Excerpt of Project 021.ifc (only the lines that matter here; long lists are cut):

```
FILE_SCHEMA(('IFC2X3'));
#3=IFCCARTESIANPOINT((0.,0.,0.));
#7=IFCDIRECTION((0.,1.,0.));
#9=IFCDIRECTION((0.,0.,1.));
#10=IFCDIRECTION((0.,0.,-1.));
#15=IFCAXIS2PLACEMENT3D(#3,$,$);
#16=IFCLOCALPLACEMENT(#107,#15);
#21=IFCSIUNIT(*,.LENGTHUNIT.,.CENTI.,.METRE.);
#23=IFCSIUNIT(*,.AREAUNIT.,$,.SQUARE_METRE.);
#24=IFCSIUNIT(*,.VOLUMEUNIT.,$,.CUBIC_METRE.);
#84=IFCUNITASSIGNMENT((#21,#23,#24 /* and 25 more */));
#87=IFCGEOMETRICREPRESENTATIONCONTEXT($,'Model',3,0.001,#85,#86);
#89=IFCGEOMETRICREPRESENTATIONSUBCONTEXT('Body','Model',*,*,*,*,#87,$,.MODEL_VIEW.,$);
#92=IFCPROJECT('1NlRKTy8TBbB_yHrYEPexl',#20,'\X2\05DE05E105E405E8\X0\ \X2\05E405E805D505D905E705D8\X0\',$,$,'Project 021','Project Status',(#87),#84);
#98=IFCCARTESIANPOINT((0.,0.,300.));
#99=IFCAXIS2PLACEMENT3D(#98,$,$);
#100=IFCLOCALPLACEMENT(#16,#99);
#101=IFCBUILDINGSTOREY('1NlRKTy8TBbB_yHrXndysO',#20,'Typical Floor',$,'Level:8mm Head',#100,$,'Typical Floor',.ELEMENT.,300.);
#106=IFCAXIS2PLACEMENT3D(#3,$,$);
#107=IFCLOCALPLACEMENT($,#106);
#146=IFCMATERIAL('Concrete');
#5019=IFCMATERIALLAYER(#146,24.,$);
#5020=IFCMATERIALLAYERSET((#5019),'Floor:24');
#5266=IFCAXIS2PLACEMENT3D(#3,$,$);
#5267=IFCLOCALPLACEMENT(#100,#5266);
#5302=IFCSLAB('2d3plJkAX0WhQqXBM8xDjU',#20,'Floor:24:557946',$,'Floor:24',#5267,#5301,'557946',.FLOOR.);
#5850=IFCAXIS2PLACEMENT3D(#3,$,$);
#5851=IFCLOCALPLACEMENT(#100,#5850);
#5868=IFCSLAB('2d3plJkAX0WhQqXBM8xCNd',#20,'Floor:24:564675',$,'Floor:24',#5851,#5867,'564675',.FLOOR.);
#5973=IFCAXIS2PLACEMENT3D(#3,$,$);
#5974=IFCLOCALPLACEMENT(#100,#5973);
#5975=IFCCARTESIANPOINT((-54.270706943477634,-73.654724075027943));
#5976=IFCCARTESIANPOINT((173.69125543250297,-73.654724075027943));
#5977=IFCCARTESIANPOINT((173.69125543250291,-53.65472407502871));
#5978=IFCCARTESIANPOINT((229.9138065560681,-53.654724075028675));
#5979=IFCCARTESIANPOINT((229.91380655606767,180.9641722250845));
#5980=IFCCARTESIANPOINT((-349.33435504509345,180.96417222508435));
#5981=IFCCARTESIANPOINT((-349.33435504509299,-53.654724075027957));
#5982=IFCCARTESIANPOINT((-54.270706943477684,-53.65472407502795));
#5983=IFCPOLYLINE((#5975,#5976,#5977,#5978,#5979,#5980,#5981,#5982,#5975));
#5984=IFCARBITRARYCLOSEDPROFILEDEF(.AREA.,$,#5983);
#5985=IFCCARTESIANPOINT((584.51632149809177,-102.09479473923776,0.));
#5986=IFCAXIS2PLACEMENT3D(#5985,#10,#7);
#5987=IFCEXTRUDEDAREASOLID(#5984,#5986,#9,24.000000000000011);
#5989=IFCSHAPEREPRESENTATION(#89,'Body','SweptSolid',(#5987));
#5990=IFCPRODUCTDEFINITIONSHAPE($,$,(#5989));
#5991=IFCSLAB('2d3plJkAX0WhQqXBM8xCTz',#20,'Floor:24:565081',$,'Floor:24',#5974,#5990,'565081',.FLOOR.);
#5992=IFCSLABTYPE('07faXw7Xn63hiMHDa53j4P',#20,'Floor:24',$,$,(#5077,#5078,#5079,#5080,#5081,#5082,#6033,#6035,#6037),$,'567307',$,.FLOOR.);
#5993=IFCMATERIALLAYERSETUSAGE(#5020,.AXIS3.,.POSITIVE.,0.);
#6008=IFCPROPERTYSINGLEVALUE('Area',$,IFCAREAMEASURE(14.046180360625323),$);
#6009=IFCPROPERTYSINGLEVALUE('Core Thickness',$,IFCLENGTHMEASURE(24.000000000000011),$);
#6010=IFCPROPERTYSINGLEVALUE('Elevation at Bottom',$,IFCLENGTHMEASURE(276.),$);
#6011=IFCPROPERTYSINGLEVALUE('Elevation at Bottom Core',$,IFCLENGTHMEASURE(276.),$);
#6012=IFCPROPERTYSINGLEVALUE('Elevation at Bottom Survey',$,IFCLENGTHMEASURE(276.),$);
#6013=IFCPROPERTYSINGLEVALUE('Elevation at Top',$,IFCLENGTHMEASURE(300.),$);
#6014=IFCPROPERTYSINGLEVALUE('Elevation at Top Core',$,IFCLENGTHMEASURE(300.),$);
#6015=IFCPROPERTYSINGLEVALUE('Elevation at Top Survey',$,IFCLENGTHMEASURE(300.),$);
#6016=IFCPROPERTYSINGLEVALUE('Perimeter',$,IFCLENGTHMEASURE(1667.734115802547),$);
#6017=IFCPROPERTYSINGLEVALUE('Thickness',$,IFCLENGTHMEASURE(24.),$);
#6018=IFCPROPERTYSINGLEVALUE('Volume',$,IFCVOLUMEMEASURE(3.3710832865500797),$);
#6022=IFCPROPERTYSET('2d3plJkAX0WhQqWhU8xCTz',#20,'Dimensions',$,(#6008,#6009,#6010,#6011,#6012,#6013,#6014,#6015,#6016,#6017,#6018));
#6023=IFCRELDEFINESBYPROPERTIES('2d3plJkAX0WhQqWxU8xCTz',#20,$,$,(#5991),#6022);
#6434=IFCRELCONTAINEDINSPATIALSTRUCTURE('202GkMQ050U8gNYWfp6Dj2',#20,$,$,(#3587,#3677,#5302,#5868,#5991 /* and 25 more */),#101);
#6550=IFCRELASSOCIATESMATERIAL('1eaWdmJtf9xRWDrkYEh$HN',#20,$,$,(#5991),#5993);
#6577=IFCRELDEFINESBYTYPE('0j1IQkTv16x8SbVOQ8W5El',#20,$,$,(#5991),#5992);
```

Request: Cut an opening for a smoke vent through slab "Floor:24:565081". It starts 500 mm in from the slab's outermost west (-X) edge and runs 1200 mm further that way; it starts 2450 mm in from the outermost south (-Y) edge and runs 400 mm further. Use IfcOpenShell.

```python
import numpy as np
import ifcopenshell
import ifcopenshell.api.feature
import ifcopenshell.api.geometry
import ifcopenshell.api.pset
import ifcopenshell.api.root
import ifcopenshell.geom
import ifcopenshell.util.element
import ifcopenshell.util.placement
import ifcopenshell.util.representation
import ifcopenshell.util.shape
import ifcopenshell.util.unit

model = ifcopenshell.open("Project 021.ifc")
unit_scale = ifcopenshell.util.unit.calculate_unit_scale(model)
area_scale = ifcopenshell.util.unit.calculate_unit_scale(model, "AREAUNIT")
volume_scale = ifcopenshell.util.unit.calculate_unit_scale(model, "VOLUMEUNIT")
settings = ifcopenshell.geom.settings()


def volume(element):
    """Net volume in cubic metres, openings subtracted."""
    shape = ifcopenshell.geom.create_shape(settings, element)
    return ifcopenshell.util.shape.get_volume(shape.geometry)


slab = model.by_guid("2d3plJkAX0WhQqXBM8xCTz")
before = volume(slab)

# Extent in the slab's own axes, in metres. The edges named are its -X and -Y sides.
slab_shape = ifcopenshell.geom.create_shape(settings, slab)
vertices = ifcopenshell.util.shape.get_vertices(slab_shape.geometry)
x_min, y_min, bottom = vertices.min(axis=0)
top = vertices[:, 2].max()

opening = ifcopenshell.api.root.create_entity(model, ifc_class="IfcOpeningElement", name="Smoke vent opening")
context = ifcopenshell.util.representation.get_context(model, "Model", "Body", "MODEL_VIEW")
width, depth = 1.2, 0.4
outline = [(0.0, 0.0), (width, 0.0), (width, depth), (0.0, depth), (0.0, 0.0)]
# Overshoot both faces by 50 mm so the cut is clean.
shape = ifcopenshell.api.geometry.add_slab_representation(
    model, context=context, depth=top - bottom + 0.1, polyline=outline
)
ifcopenshell.api.geometry.assign_representation(model, product=opening, representation=shape)

matrix = ifcopenshell.util.placement.get_local_placement(slab.ObjectPlacement)
matrix[:, 3] = matrix @ np.append(np.array([x_min + 0.5, y_min + 2.45, bottom - 0.05]) / unit_scale, 1.0)
ifcopenshell.api.geometry.edit_object_placement(model, product=opening, matrix=matrix, is_si=False)
ifcopenshell.api.feature.add_feature(model, feature=opening, element=slab)

after = volume(slab)

# Update the slab's stored quantities.
pset = model.by_id(ifcopenshell.util.element.get_pset(slab, "Dimensions", should_inherit=False)["id"])
ifcopenshell.api.pset.edit_pset(model, pset=pset, properties={
    "Area": model.create_entity("IfcAreaMeasure", after / (top - bottom) / area_scale),
    "Volume": model.create_entity("IfcVolumeMeasure", after / volume_scale),
})

print(f"slab volume {before:.3f} -> {after:.3f} m3")

model.write("Project 021-out.ifc")
```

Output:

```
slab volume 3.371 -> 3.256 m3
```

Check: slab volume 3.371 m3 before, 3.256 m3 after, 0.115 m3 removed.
